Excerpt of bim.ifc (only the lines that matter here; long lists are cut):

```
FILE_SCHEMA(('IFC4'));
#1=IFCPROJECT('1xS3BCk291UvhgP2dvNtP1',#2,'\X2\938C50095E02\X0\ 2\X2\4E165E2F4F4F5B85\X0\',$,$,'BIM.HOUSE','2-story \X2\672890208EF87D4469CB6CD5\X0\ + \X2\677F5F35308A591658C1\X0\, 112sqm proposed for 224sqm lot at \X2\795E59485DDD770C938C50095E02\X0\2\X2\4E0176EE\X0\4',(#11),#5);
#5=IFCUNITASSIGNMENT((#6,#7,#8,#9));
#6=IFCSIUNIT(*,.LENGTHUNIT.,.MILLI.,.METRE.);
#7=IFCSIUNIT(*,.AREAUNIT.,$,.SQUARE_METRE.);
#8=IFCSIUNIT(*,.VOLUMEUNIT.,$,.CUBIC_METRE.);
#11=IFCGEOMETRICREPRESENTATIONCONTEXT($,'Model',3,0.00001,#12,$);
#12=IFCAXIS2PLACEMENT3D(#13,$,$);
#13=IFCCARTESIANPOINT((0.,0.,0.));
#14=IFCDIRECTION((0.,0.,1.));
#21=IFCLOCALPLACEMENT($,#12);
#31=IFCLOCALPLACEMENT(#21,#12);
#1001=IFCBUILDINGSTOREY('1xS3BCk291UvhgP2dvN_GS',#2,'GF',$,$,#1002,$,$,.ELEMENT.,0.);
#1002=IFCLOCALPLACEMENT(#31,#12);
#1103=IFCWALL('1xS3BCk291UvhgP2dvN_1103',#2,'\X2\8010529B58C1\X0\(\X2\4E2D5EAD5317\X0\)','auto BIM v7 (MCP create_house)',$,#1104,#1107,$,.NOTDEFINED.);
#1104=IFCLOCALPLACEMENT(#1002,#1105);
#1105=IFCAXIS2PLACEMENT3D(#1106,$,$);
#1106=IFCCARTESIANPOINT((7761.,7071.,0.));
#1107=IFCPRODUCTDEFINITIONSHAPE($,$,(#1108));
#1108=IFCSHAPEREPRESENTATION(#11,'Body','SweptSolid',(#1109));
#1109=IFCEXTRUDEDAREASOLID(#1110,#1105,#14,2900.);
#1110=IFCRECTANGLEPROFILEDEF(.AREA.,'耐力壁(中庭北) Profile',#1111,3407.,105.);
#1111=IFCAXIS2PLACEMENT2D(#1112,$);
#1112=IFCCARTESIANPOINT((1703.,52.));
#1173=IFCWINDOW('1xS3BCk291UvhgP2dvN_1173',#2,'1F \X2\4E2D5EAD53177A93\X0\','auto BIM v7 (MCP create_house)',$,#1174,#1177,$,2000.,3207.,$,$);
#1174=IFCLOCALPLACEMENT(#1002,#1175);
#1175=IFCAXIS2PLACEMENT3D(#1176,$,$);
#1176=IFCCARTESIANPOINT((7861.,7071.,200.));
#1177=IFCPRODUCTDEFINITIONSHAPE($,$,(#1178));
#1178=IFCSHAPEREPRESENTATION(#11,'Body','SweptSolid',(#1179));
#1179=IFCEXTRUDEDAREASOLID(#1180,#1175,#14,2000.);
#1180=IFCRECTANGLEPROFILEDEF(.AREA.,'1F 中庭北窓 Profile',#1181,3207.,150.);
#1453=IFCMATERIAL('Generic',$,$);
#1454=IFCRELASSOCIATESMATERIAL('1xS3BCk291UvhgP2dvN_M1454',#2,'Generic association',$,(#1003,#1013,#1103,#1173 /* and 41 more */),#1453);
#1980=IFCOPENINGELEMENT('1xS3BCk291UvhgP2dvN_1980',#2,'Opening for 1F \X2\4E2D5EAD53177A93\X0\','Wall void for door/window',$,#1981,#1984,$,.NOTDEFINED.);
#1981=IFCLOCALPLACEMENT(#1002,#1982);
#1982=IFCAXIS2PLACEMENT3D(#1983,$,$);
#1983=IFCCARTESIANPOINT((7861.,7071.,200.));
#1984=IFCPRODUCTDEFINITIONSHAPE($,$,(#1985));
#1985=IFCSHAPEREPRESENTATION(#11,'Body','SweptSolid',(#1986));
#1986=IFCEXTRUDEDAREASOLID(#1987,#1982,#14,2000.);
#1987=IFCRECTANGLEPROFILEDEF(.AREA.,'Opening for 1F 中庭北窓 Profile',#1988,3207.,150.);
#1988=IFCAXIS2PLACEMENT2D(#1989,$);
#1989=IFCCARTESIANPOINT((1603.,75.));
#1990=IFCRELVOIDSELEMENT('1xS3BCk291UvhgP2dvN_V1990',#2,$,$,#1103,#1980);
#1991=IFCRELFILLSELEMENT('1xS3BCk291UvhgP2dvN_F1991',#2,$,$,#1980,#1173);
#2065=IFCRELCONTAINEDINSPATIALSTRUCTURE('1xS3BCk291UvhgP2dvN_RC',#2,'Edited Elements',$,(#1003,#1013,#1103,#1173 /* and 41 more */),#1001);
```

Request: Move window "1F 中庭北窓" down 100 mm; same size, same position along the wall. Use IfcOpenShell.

```python
import numpy as np
import ifcopenshell
import ifcopenshell.api.geometry
import ifcopenshell.util.placement
import ifcopenshell.util.unit

model = ifcopenshell.open("bim.ifc")
unit_scale = ifcopenshell.util.unit.calculate_unit_scale(model)

window = model.by_guid("1xS3BCk291UvhgP2dvN_1173")
opening = window.FillsVoids[0].RelatingOpeningElement
dz = -0.1 / unit_scale

shift = np.array([0.0, 0.0, dz])
# The window is not placed relative to its opening, so move both.
for product in (opening, window):
    matrix = ifcopenshell.util.placement.get_local_placement(product.ObjectPlacement)
    matrix[:3, 3] += shift
    ifcopenshell.api.geometry.edit_object_placement(model, product=product, matrix=matrix, is_si=False)

print(f"moved by {dz * unit_scale:+.3f} m")

model.write("bim-out.ifc")
```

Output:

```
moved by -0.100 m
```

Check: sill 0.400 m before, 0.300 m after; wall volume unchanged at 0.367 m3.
